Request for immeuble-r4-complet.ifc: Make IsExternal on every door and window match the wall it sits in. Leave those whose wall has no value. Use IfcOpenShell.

First a look at what the model holds.

```python
import ifcopenshell
import ifcopenshell.util.element

model = ifcopenshell.open("immeuble-r4-complet.ifc")
print(model.schema)
seen = {}
for e in model.by_type("IfcDoor") + model.by_type("IfcWindow"):
    if not e.FillsVoids:
        continue
    host = e.FillsVoids[0].RelatingOpeningElement.VoidsElements[0].RelatingBuildingElement
    own = ifcopenshell.util.element.get_pset(e, f"Pset_{e.is_a()[3:].removesuffix('StandardCase')}Common", "IsExternal")
    wall = ifcopenshell.util.element.get_pset(host, "Pset_WallCommon", "IsExternal")
    seen[e.is_a(), own, wall] = seen.get((e.is_a(), own, wall), 0) + 1
for (cls, own, wall), count in sorted(seen.items(), key=str):
    print(count, cls, "IsExternal:", own, "| host wall:", wall)
```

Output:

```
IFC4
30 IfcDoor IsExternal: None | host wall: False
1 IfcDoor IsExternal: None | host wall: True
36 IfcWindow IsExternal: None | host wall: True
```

```python
import ifcopenshell
import ifcopenshell.api.pset
import ifcopenshell.util.element

model = ifcopenshell.open("immeuble-r4-complet.ifc")

count = 0
for ifc_class, pset_name in (("IfcDoor", "Pset_DoorCommon"), ("IfcWindow", "Pset_WindowCommon")):
    for e in model.by_type(ifc_class):
        if not e.FillsVoids:
            continue
        host = e.FillsVoids[0].RelatingOpeningElement.VoidsElements[0].RelatingBuildingElement
        external = ifcopenshell.util.element.get_pset(host, "Pset_WallCommon", "IsExternal")
        if external is None or ifcopenshell.util.element.get_pset(e, pset_name, "IsExternal") == external:
            continue
        pset = ifcopenshell.api.pset.add_pset(model, product=e, name=pset_name)
        ifcopenshell.api.pset.edit_pset(model, pset=pset, properties={"IsExternal": external})
        count += 1

print(count, "updated")

model.write("immeuble-r4-complet-out.ifc")
```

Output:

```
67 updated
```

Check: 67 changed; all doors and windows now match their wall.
